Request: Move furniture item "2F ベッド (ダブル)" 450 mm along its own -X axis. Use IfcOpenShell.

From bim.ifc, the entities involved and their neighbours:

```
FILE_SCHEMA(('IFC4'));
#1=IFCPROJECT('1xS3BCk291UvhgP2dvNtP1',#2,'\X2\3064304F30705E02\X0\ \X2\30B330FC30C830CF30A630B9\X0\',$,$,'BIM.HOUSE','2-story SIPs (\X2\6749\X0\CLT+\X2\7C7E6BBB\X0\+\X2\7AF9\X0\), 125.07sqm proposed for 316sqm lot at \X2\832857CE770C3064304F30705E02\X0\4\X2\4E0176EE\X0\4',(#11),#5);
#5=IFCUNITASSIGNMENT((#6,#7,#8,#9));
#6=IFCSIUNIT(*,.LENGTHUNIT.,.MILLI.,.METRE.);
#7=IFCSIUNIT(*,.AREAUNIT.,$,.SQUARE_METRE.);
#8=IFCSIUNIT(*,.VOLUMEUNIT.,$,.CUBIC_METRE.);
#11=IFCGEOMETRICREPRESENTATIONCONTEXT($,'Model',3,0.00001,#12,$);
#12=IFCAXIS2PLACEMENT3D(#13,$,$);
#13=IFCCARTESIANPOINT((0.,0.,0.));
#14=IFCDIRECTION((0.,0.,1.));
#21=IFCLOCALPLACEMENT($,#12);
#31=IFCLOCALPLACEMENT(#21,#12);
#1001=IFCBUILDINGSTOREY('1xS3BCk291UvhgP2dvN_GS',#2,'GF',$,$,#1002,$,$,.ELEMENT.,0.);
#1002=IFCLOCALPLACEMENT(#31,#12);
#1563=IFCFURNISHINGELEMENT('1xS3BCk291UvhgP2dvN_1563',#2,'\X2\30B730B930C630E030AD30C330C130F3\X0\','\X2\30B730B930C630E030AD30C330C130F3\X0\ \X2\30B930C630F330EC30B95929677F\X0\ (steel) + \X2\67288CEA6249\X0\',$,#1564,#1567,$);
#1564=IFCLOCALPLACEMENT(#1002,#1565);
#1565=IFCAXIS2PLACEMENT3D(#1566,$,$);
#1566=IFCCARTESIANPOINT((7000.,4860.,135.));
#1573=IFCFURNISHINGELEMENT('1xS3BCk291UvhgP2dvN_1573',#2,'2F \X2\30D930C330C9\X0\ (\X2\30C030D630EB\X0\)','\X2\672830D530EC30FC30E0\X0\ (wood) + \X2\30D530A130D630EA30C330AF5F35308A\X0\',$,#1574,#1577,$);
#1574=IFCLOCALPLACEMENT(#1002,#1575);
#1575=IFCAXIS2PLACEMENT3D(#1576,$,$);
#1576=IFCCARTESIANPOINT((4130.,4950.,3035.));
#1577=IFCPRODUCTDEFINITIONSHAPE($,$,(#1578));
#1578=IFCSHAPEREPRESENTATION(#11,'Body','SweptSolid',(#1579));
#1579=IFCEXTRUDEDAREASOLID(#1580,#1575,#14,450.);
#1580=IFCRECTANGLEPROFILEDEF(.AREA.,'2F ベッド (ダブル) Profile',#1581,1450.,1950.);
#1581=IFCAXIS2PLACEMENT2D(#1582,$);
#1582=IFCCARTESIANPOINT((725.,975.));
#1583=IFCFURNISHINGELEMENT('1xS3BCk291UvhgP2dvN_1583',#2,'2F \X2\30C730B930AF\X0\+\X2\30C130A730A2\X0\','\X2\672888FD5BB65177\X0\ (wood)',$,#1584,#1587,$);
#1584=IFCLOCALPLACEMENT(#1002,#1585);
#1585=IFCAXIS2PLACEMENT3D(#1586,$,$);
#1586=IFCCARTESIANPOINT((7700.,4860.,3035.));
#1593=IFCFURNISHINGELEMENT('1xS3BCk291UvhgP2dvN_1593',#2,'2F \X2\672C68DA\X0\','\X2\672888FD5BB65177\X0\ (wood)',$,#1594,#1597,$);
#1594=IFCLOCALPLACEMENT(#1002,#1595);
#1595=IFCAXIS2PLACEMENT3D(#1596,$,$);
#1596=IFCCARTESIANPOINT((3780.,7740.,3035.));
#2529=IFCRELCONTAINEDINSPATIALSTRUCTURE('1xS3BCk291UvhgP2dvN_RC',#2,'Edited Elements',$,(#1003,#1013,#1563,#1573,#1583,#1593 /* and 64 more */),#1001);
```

```python
import ifcopenshell
import ifcopenshell.api.geometry
import ifcopenshell.util.placement
import ifcopenshell.util.unit

model = ifcopenshell.open("bim.ifc")
unit_scale = ifcopenshell.util.unit.calculate_unit_scale(model)

item = model.by_id(1573)
matrix = ifcopenshell.util.placement.get_local_placement(item.ObjectPlacement)
matrix[:3, 3] -= matrix[:3, 0] * 0.45 / unit_scale
ifcopenshell.api.geometry.edit_object_placement(model, product=item, matrix=matrix, is_si=False)

print(ifcopenshell.util.placement.get_local_placement(item.ObjectPlacement).round(3) + 0.0)

model.write("bim-out.ifc")
```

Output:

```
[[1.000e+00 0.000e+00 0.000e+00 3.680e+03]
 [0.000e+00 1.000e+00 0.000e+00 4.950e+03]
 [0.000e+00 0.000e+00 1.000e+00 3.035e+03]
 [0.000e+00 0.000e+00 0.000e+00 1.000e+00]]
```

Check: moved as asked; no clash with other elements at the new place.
